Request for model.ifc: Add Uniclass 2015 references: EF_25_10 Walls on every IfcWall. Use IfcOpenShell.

First a look at what the model holds.

```python
import ifcopenshell

model = ifcopenshell.open("model.ifc")
print(model.schema)
print("classifications:", [c.Name for c in model.by_type("IfcClassification")])
for ifc_class in ("IfcDoor", "IfcRoof", "IfcStair", "IfcWall", "IfcWindow"):
    print(ifc_class, len(model.by_type(ifc_class)))
```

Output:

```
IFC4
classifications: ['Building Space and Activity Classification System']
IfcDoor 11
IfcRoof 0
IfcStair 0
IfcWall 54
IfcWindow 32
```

```python
import ifcopenshell
import ifcopenshell.api.classification

model = ifcopenshell.open("model.ifc")

system = ifcopenshell.api.classification.add_classification(model, classification="Uniclass 2015")

codes = {
    "IfcWall": ("EF_25_10", "Walls"),
}
for ifc_class, (code, name) in codes.items():
    products = model.by_type(ifc_class)
    ifcopenshell.api.classification.add_reference(
        model, products=products, classification=system, identification=code, name=name
    )
    print(code, len(products))

model.write("model_edited.ifc")
```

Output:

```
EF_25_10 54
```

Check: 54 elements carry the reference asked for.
